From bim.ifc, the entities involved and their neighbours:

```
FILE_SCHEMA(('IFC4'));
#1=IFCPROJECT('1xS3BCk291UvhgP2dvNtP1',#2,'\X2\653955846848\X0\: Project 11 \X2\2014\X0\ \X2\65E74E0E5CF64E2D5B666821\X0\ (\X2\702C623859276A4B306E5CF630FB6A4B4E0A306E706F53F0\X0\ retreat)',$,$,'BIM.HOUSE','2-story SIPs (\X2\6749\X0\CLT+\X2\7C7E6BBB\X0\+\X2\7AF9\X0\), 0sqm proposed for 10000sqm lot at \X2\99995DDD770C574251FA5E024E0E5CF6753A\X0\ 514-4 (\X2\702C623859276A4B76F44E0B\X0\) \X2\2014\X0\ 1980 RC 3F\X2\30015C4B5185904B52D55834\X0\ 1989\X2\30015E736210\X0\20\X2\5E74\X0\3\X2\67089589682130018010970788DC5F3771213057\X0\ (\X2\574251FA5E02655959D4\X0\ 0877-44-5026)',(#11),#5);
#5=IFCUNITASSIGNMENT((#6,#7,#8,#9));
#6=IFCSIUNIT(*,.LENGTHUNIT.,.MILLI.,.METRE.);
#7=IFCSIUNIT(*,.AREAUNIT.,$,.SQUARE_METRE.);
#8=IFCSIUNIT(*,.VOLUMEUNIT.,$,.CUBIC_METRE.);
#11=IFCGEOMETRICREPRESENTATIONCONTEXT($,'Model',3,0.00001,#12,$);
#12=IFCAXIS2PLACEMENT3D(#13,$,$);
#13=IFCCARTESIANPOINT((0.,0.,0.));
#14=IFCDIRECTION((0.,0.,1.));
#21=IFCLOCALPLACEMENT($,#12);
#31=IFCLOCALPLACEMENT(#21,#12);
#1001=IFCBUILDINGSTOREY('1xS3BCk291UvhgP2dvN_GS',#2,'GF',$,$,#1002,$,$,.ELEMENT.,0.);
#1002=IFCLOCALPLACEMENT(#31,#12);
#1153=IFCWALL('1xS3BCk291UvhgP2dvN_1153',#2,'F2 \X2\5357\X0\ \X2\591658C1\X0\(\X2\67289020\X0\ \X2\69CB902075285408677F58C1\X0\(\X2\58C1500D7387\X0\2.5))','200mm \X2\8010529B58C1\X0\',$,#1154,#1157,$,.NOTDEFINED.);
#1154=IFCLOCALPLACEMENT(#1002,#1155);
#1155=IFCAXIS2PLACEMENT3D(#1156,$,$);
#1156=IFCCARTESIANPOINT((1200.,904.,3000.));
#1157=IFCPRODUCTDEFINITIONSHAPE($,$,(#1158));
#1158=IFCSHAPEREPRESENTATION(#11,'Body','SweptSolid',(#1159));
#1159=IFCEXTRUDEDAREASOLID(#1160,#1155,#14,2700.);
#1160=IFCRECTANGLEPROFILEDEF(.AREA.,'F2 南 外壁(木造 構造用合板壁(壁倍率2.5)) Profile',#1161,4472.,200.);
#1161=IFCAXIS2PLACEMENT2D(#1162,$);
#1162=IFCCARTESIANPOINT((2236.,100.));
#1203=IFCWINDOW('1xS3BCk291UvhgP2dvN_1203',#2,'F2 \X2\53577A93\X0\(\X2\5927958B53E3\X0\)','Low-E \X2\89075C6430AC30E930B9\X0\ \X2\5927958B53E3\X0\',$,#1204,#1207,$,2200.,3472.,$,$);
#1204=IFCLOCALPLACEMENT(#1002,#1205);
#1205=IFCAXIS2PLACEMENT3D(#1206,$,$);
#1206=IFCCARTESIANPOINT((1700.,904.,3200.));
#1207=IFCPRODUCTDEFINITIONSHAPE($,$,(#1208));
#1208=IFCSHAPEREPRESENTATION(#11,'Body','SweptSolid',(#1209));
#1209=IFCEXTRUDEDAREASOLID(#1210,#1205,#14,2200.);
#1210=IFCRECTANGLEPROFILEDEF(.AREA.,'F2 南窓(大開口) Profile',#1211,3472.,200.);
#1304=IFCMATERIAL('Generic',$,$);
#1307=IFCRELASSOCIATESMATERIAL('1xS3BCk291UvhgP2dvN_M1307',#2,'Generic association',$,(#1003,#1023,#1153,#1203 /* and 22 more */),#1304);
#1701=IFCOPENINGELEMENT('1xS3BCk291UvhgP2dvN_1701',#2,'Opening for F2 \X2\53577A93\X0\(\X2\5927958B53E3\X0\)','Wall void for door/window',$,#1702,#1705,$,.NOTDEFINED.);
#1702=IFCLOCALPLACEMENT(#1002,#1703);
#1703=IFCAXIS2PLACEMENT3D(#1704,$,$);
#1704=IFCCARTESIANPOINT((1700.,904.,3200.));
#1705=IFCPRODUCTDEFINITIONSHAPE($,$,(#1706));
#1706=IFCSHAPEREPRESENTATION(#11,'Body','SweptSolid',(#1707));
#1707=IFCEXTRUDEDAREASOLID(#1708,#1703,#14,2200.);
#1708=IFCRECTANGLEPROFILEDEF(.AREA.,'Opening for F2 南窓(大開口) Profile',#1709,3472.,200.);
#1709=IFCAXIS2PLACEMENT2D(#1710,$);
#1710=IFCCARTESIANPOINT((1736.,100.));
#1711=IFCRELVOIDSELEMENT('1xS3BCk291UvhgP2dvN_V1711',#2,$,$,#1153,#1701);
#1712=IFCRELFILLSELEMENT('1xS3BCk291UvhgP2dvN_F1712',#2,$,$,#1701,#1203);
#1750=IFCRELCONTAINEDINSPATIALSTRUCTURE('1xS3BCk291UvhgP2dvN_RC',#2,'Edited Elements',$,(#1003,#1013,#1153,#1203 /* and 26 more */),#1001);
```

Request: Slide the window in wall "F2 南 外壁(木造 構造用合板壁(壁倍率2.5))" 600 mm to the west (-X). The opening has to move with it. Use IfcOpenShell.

```python
import ifcopenshell
import ifcopenshell.api.geometry
import ifcopenshell.util.placement
import ifcopenshell.util.unit

model = ifcopenshell.open("bim.ifc")
unit_scale = ifcopenshell.util.unit.calculate_unit_scale(model)

window = model.by_guid("1xS3BCk291UvhgP2dvN_1203")
opening = window.FillsVoids[0].RelatingOpeningElement
wall = opening.VoidsElements[0].RelatingBuildingElement

wall_matrix = ifcopenshell.util.placement.get_local_placement(wall.ObjectPlacement)
shift = wall_matrix[:3, 0] * -0.6 / unit_scale
before = ifcopenshell.util.placement.get_local_placement(window.ObjectPlacement)[:3, 3].copy()

# The window is not placed relative to its opening, so move both.
for product in (opening, window):
    matrix = ifcopenshell.util.placement.get_local_placement(product.ObjectPlacement)
    matrix[:3, 3] += shift
    ifcopenshell.api.geometry.edit_object_placement(model, product=product, matrix=matrix, is_si=False)

after = ifcopenshell.util.placement.get_local_placement(window.ObjectPlacement)[:3, 3]
print("window moved by", (after - before).round(3) + 0.0)

model.write("bim_updated.ifc")
```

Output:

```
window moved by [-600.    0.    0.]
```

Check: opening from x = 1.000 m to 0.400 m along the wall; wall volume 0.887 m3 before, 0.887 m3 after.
